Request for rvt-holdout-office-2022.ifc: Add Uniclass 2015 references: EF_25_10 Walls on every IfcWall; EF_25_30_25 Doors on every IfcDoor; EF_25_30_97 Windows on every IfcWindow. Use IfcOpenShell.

First a look at what the model holds.

```python
import ifcopenshell

model = ifcopenshell.open("rvt-holdout-office-2022.ifc")
print(model.schema)
print("classifications:", [c.Name for c in model.by_type("IfcClassification")])
for ifc_class in ("IfcDoor", "IfcRoof", "IfcStair", "IfcWall", "IfcWindow"):
    print(ifc_class, len(model.by_type(ifc_class)))
```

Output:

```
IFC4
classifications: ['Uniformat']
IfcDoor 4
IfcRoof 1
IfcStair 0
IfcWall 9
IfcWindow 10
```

```python
import ifcopenshell
import ifcopenshell.api.classification

model = ifcopenshell.open("rvt-holdout-office-2022.ifc")

system = ifcopenshell.api.classification.add_classification(model, classification="Uniclass 2015")

codes = {
    "IfcWall": ("EF_25_10", "Walls"),
    "IfcDoor": ("EF_25_30_25", "Doors"),
    "IfcWindow": ("EF_25_30_97", "Windows"),
}
for ifc_class, (code, name) in codes.items():
    products = model.by_type(ifc_class)
    ifcopenshell.api.classification.add_reference(
        model, products=products, classification=system, identification=code, name=name
    )
    print(code, len(products))

model.write("rvt-holdout-office-2022_v2.ifc")
```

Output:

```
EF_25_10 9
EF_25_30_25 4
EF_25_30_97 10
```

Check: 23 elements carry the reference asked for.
